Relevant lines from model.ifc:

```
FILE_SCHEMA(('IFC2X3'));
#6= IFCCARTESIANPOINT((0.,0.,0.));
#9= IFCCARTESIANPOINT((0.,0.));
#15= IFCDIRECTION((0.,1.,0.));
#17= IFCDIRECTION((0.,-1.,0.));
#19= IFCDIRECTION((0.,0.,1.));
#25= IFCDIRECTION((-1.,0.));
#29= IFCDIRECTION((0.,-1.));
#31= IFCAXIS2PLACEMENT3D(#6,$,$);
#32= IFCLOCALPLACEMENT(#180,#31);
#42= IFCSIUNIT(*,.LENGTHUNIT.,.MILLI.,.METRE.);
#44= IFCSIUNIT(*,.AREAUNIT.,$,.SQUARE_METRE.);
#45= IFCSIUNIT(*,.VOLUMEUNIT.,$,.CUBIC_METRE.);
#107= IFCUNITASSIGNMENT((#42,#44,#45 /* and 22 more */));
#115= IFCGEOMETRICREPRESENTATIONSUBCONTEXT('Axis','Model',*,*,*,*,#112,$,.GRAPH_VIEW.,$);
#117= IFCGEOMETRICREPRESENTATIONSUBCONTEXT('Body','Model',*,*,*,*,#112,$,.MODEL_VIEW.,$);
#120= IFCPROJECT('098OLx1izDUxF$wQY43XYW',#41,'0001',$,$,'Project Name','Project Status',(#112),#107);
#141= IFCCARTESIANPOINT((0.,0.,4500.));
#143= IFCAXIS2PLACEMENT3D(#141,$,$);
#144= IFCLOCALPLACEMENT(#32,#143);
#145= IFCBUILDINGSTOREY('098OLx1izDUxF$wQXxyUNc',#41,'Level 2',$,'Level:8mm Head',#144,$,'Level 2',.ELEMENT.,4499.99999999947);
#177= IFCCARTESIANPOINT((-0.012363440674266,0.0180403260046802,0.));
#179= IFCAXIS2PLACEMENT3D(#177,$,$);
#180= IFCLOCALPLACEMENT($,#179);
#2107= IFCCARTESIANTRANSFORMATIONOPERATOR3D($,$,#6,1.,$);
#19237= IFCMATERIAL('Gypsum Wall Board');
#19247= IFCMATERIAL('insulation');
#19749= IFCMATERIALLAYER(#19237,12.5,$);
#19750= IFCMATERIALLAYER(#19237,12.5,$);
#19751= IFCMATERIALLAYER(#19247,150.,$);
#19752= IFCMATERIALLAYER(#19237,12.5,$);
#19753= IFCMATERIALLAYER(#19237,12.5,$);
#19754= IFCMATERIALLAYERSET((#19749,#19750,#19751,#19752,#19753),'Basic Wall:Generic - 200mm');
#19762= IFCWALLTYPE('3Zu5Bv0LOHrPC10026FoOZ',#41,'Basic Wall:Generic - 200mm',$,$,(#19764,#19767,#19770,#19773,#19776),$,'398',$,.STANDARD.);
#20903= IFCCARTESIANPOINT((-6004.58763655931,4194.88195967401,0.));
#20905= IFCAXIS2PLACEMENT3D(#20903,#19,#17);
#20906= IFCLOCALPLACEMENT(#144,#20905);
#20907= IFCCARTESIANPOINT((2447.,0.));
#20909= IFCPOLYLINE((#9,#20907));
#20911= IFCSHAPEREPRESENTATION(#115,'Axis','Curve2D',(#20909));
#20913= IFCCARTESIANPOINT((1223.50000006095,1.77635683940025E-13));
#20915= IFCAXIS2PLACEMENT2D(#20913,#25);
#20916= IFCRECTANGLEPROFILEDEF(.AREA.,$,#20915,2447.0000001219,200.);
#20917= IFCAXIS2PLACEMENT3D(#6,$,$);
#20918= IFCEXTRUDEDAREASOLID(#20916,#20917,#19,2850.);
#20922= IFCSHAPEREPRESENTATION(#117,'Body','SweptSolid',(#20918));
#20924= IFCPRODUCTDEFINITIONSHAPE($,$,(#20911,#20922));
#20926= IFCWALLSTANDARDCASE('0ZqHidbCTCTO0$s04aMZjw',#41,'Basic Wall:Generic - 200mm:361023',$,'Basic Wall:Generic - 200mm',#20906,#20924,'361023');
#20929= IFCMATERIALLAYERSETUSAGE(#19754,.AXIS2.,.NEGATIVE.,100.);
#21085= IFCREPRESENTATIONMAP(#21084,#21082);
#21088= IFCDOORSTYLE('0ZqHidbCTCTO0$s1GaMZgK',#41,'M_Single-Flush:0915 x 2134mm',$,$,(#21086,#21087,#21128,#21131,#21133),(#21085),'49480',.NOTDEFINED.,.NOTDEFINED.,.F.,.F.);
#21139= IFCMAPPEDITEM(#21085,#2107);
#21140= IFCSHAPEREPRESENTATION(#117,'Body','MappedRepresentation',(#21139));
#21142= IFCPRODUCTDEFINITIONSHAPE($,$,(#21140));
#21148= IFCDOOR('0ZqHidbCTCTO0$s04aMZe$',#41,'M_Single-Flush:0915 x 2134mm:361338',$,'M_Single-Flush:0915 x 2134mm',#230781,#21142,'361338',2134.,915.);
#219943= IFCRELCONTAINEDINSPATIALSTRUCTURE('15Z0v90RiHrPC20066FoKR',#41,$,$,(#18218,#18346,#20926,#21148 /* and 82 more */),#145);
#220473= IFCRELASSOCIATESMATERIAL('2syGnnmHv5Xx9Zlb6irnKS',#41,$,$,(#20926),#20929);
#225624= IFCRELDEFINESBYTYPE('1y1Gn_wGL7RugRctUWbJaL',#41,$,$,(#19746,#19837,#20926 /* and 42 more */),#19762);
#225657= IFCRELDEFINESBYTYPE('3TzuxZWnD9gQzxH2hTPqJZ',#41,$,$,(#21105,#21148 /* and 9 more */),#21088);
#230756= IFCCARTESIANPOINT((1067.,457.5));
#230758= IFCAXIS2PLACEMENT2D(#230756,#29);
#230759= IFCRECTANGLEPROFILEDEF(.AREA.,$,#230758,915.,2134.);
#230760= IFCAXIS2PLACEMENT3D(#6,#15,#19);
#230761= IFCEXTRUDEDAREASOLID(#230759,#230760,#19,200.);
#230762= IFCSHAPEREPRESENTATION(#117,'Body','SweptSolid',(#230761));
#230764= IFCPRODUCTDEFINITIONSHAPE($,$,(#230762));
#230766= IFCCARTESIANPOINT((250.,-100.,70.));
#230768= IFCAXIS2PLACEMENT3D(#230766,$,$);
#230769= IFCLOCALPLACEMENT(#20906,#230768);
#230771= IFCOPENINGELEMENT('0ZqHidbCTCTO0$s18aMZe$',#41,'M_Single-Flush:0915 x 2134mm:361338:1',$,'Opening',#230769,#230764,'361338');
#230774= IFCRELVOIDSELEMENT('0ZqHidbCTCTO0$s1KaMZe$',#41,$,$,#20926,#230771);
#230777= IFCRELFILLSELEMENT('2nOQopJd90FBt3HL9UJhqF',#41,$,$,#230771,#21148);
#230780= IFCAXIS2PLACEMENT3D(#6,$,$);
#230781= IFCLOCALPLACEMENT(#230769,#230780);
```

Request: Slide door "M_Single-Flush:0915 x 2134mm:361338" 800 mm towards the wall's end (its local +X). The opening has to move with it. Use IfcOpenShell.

```python
import ifcopenshell
import ifcopenshell.api.geometry
import ifcopenshell.util.placement

model = ifcopenshell.open("model.ifc")

door = model.by_guid("0ZqHidbCTCTO0$s04aMZe$")
opening = door.FillsVoids[0].RelatingOpeningElement
wall = opening.VoidsElements[0].RelatingBuildingElement

wall_matrix = ifcopenshell.util.placement.get_local_placement(wall.ObjectPlacement)
shift = wall_matrix[:3, 0] * 800.0
before = ifcopenshell.util.placement.get_local_placement(door.ObjectPlacement)[:3, 3].copy()

# The door is placed relative to its opening, so it follows when the opening moves.
matrix = ifcopenshell.util.placement.get_local_placement(opening.ObjectPlacement)
matrix[:3, 3] += shift
ifcopenshell.api.geometry.edit_object_placement(
    model, product=opening, matrix=matrix, is_si=False, should_transform_children=True
)

after = ifcopenshell.util.placement.get_local_placement(door.ObjectPlacement)[:3, 3]
print("door moved by", (after - before).round(3) + 0.0)

model.write("model_edited.ifc")
```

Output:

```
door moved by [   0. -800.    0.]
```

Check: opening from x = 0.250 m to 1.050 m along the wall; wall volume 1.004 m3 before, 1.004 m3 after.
